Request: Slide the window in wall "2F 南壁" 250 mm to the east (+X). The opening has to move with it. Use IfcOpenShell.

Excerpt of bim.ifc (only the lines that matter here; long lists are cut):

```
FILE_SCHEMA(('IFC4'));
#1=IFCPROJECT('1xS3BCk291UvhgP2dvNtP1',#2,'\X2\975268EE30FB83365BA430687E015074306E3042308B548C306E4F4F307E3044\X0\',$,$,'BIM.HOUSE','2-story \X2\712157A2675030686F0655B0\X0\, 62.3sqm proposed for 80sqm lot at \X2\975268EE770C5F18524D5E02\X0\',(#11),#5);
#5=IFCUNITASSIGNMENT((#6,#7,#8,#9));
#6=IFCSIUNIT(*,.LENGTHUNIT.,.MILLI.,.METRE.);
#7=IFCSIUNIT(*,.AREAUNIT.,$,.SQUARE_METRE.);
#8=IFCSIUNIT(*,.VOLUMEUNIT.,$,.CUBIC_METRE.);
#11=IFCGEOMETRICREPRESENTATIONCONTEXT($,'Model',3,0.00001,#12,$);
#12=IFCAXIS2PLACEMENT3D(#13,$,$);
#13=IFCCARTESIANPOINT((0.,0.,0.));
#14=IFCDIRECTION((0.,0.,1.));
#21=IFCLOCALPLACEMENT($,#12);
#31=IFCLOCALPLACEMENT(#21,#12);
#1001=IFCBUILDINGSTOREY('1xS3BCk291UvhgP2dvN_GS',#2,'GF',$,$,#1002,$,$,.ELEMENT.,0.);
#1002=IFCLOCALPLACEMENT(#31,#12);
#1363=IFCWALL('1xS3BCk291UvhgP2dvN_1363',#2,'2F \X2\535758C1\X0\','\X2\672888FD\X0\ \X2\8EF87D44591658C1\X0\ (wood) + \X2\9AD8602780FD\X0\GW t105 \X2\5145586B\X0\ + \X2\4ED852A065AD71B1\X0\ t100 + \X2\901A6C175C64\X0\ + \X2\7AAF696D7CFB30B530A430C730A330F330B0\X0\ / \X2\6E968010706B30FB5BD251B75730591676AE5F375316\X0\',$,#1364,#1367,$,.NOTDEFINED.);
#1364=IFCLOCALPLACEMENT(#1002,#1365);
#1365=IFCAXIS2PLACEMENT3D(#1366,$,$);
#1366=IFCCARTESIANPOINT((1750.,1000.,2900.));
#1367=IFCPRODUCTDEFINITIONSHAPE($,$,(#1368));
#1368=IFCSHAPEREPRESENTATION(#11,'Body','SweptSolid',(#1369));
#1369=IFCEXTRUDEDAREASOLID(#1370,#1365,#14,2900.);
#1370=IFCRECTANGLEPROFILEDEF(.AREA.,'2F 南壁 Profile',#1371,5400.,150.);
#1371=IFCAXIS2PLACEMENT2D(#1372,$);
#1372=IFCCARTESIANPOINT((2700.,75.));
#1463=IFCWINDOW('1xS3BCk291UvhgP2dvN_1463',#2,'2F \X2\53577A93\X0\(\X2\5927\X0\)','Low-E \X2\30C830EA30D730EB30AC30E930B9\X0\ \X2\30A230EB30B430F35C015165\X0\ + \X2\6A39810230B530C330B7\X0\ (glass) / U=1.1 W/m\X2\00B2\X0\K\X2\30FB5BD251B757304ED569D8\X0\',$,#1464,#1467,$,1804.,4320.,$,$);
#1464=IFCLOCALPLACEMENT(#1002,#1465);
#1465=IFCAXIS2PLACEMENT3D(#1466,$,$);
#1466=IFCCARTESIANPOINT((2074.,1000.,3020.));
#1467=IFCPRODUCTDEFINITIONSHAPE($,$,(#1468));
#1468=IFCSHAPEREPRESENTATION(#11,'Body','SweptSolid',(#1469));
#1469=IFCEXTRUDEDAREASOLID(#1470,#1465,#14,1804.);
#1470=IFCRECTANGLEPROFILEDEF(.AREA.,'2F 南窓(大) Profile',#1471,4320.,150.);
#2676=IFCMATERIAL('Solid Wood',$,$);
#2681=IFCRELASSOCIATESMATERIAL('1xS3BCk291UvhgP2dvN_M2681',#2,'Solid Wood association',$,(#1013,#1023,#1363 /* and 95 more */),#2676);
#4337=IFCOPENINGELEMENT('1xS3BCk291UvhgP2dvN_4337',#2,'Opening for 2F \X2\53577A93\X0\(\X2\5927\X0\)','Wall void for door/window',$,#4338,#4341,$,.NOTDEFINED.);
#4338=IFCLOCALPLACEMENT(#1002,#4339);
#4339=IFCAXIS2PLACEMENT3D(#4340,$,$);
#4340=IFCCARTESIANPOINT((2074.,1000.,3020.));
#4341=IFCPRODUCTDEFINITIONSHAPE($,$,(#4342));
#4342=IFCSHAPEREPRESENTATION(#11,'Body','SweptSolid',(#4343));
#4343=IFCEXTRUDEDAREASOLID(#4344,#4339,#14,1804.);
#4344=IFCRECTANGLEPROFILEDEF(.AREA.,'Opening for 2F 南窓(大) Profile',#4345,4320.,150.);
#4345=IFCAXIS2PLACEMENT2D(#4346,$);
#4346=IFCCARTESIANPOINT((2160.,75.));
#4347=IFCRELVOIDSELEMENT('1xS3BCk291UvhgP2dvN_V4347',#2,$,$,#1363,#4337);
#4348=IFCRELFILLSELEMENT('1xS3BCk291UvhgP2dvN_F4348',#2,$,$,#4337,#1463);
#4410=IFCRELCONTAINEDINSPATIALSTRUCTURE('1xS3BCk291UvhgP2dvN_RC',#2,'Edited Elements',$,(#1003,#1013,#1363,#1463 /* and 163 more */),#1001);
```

```python
import ifcopenshell
import ifcopenshell.api.geometry
import ifcopenshell.util.placement
import ifcopenshell.util.unit

model = ifcopenshell.open("bim.ifc")
unit_scale = ifcopenshell.util.unit.calculate_unit_scale(model)

window = model.by_guid("1xS3BCk291UvhgP2dvN_1463")
opening = window.FillsVoids[0].RelatingOpeningElement
wall = opening.VoidsElements[0].RelatingBuildingElement

wall_matrix = ifcopenshell.util.placement.get_local_placement(wall.ObjectPlacement)
shift = wall_matrix[:3, 0] * 0.25 / unit_scale
before = ifcopenshell.util.placement.get_local_placement(window.ObjectPlacement)[:3, 3].copy()

# The window is not placed relative to its opening, so move both.
for product in (opening, window):
    matrix = ifcopenshell.util.placement.get_local_placement(product.ObjectPlacement)
    matrix[:3, 3] += shift
    ifcopenshell.api.geometry.edit_object_placement(model, product=product, matrix=matrix, is_si=False)

after = ifcopenshell.util.placement.get_local_placement(window.ObjectPlacement)[:3, 3]
print("window moved by", (after - before).round(3) + 0.0)

model.write("bim_edited.ifc")
```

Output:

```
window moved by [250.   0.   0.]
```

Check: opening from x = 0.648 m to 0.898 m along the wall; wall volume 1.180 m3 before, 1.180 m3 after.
